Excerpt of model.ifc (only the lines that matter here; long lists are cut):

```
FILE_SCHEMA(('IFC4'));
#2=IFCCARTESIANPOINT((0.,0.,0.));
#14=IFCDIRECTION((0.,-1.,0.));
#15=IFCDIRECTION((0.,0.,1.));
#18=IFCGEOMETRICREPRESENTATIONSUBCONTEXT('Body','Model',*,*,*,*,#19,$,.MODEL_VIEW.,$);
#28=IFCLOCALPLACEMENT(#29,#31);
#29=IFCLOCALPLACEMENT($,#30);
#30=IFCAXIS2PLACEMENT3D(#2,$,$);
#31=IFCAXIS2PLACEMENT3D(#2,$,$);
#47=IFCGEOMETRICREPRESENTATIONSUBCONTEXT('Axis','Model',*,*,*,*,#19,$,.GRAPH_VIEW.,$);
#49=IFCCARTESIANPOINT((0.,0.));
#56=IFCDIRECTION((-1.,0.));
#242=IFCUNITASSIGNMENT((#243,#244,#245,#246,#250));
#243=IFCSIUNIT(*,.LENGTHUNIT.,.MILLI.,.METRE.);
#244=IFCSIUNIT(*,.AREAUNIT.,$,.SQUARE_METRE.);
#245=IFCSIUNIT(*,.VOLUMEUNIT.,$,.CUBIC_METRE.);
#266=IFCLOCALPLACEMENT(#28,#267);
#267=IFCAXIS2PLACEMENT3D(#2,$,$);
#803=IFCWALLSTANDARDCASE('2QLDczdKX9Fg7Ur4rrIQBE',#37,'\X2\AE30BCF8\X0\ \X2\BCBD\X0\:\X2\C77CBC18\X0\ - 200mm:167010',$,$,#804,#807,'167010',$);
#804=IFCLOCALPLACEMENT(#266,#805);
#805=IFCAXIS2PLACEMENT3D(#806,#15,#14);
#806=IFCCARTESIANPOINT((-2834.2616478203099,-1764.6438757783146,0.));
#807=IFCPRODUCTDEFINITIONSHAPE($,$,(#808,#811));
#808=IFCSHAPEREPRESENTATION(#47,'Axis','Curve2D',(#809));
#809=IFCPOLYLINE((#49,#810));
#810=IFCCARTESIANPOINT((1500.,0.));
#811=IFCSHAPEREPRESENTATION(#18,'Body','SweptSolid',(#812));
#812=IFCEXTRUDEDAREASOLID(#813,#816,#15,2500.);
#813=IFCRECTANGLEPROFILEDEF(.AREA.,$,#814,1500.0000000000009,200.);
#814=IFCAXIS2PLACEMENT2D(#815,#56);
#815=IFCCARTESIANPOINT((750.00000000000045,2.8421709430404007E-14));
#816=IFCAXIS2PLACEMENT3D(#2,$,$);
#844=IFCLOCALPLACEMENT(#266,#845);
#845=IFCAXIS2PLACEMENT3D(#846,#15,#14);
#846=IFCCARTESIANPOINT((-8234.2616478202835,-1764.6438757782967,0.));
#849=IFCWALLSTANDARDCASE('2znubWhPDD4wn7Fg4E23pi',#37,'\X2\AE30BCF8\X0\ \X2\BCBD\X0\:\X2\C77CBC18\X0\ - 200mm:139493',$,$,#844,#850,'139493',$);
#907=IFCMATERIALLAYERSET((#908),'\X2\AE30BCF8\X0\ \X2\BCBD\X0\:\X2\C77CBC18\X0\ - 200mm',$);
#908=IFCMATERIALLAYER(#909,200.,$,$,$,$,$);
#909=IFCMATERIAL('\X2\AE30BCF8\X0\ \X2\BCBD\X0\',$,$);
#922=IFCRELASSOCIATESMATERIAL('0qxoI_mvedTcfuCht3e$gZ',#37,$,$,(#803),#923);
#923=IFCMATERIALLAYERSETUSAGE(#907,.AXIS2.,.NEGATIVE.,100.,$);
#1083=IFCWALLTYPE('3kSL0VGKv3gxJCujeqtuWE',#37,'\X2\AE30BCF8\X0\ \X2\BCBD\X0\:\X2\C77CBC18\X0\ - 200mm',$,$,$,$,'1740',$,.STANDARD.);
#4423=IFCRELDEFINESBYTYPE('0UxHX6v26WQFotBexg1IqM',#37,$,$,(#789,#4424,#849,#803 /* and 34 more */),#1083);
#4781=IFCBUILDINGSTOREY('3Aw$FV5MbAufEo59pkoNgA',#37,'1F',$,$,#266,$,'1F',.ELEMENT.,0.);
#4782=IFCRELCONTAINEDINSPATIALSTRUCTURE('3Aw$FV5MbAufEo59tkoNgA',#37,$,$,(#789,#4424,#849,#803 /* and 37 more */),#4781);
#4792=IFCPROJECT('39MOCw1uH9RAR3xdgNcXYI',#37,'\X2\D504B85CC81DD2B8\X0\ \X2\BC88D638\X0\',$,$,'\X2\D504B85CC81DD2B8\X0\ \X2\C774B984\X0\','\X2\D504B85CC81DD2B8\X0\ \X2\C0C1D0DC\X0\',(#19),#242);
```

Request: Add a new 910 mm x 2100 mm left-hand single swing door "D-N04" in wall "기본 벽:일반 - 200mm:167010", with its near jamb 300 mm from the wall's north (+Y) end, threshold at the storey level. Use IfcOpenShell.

```python
import numpy as np
import ifcopenshell
import ifcopenshell.api.feature
import ifcopenshell.api.geometry
import ifcopenshell.api.root
import ifcopenshell.api.spatial
import ifcopenshell.geom
import ifcopenshell.util.element
import ifcopenshell.util.placement
import ifcopenshell.util.representation
import ifcopenshell.util.shape
import ifcopenshell.util.unit

model = ifcopenshell.open("model.ifc")
unit_scale = ifcopenshell.util.unit.calculate_unit_scale(model)
settings = ifcopenshell.geom.settings()


def volume(element):
    """Net volume in cubic metres, openings subtracted."""
    shape = ifcopenshell.geom.create_shape(settings, element)
    return ifcopenshell.util.shape.get_volume(shape.geometry)


wall = model.by_id(803)
storey = ifcopenshell.util.element.get_container(wall, ifc_class="IfcBuildingStorey")
context = ifcopenshell.util.representation.get_context(model, "Model", "Body", "MODEL_VIEW")
before = volume(wall)

width, height, from_end, sill = 0.91, 2.1, 0.3, 0.0  # metres

# The wall runs along its own X axis, and the end named is its -X end.
wall_shape = ifcopenshell.geom.create_shape(settings, wall)
x, y, z = ifcopenshell.util.shape.get_vertices(wall_shape.geometry).T
start = x.min() + from_end
face, thickness = float(y.min()), float(y.max() - y.min())
wall_matrix = ifcopenshell.util.placement.get_local_placement(wall.ObjectPlacement)
level = ifcopenshell.util.placement.get_local_placement(storey.ObjectPlacement)[2, 3]


def in_wall(x, y):
    """Placement at x, y metres in the wall's axes, at sill height."""
    matrix = wall_matrix.copy()
    matrix[:, 3] = wall_matrix @ np.array([x / unit_scale, y / unit_scale, 0.0, 1.0])
    matrix[2, 3] = level + sill / unit_scale
    return matrix


# Opening: a box that overshoots both wall faces by 50 mm.
opening = ifcopenshell.api.root.create_entity(model, ifc_class="IfcOpeningElement", predefined_type="OPENING")
box = ifcopenshell.api.geometry.add_wall_representation(
    model, context=context, length=width, height=height, thickness=thickness + 0.1
)
ifcopenshell.api.geometry.assign_representation(model, product=opening, representation=box)
ifcopenshell.api.geometry.edit_object_placement(model, product=opening, matrix=in_wall(start, face - 0.05), is_si=False)
ifcopenshell.api.feature.add_feature(model, feature=opening, element=wall)

door = ifcopenshell.api.root.create_entity(model, ifc_class="IfcDoor", name="D-N04", predefined_type="DOOR")
door.OverallWidth, door.OverallHeight = width / unit_scale, height / unit_scale
door.OperationType = "SINGLE_SWING_LEFT"
body = ifcopenshell.api.geometry.add_door_representation(
    model,
    context=context,
    overall_width=door.OverallWidth,
    overall_height=door.OverallHeight,
    operation_type="SINGLE_SWING_LEFT",
    lining_properties={"LiningDepth": thickness / unit_scale, "ThresholdDepth": thickness / unit_scale},
)
ifcopenshell.api.geometry.assign_representation(model, product=door, representation=body)
ifcopenshell.api.spatial.assign_container(model, products=[door], relating_structure=storey)
ifcopenshell.api.feature.add_filling(model, opening=opening, element=door)

# The lining spans the wall, so the door starts at the wall face.
ifcopenshell.api.geometry.edit_object_placement(model, product=door, matrix=in_wall(start, face), is_si=False)

after = volume(wall)

print(f"wall volume {before:.3f} -> {after:.3f} m3")

model.write("model-out.ifc")
```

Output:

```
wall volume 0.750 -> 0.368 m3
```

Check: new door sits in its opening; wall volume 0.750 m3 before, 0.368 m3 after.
